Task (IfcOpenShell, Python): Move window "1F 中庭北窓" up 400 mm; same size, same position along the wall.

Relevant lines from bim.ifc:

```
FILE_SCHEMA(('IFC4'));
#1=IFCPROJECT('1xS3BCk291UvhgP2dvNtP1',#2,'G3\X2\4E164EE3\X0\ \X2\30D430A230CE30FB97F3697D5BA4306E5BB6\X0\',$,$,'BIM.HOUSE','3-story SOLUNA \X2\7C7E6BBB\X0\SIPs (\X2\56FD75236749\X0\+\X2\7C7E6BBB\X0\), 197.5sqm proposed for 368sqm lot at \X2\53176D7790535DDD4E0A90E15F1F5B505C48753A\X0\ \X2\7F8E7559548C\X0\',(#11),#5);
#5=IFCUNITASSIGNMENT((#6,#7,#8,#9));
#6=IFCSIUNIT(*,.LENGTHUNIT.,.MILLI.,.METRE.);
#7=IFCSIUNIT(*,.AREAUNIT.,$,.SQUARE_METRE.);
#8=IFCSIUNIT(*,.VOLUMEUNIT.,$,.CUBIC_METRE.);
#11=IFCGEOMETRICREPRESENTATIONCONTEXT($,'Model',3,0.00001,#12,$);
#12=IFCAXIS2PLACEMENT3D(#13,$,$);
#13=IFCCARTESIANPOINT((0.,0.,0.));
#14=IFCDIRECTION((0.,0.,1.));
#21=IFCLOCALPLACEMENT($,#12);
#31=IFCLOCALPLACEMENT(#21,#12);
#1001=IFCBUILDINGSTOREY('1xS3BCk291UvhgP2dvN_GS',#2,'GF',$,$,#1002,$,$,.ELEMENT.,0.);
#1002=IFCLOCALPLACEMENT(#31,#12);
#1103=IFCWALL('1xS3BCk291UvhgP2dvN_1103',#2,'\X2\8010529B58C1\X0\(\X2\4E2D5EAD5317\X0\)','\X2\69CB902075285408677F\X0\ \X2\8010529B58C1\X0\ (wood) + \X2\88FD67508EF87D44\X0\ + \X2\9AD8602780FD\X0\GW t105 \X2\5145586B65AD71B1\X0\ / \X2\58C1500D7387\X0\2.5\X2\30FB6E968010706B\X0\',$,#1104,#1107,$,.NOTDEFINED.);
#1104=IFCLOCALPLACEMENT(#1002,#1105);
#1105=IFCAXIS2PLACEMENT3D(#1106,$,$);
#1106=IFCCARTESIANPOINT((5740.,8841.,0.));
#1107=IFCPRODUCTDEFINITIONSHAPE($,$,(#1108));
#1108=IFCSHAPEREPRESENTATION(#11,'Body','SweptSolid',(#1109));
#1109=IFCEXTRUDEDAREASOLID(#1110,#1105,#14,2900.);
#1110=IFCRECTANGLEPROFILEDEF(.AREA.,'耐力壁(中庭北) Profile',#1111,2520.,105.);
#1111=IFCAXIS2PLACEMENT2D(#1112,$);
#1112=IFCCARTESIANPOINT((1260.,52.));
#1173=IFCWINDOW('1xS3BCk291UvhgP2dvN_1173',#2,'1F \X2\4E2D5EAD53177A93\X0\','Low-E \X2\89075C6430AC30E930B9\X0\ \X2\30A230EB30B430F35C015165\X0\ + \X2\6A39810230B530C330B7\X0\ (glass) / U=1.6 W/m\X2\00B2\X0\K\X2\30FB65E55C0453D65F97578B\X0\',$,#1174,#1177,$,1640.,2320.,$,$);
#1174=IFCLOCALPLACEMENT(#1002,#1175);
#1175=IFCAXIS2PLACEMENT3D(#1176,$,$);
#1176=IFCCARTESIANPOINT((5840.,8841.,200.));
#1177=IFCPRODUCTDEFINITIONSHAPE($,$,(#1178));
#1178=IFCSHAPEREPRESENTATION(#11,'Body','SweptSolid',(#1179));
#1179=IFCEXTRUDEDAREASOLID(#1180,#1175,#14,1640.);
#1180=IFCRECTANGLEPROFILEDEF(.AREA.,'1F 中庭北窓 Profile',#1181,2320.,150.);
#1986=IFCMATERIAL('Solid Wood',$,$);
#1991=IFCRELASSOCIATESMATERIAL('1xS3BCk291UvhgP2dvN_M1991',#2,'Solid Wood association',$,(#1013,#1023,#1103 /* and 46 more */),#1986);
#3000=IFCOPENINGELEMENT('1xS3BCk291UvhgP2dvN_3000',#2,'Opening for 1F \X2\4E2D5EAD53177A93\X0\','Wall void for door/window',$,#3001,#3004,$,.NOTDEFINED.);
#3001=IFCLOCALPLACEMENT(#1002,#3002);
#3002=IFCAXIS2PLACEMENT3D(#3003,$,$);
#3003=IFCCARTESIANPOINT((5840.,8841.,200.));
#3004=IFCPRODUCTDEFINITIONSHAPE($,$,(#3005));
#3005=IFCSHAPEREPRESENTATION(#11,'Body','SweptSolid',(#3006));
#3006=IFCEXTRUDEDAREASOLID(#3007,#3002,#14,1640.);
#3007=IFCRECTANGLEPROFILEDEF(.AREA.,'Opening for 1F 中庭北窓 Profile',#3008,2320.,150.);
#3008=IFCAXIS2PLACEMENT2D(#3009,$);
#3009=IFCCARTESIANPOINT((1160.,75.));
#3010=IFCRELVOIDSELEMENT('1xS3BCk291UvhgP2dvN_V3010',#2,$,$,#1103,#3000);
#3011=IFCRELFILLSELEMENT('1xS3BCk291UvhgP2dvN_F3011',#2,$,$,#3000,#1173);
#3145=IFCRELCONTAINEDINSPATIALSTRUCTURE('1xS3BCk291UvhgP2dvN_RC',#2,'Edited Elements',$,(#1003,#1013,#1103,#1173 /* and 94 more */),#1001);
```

```python
import numpy as np
import ifcopenshell
import ifcopenshell.api.geometry
import ifcopenshell.util.placement
import ifcopenshell.util.unit

model = ifcopenshell.open("bim.ifc")
unit_scale = ifcopenshell.util.unit.calculate_unit_scale(model)

window = model.by_guid("1xS3BCk291UvhgP2dvN_1173")
opening = window.FillsVoids[0].RelatingOpeningElement
dz = 0.4 / unit_scale

shift = np.array([0.0, 0.0, dz])
# The window is not placed relative to its opening, so move both.
for product in (opening, window):
    matrix = ifcopenshell.util.placement.get_local_placement(product.ObjectPlacement)
    matrix[:3, 3] += shift
    ifcopenshell.api.geometry.edit_object_placement(model, product=product, matrix=matrix, is_si=False)

print(f"moved by {dz * unit_scale:+.3f} m")

model.write("bim_updated.ifc")
```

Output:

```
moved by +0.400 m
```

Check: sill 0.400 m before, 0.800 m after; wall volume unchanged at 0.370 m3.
